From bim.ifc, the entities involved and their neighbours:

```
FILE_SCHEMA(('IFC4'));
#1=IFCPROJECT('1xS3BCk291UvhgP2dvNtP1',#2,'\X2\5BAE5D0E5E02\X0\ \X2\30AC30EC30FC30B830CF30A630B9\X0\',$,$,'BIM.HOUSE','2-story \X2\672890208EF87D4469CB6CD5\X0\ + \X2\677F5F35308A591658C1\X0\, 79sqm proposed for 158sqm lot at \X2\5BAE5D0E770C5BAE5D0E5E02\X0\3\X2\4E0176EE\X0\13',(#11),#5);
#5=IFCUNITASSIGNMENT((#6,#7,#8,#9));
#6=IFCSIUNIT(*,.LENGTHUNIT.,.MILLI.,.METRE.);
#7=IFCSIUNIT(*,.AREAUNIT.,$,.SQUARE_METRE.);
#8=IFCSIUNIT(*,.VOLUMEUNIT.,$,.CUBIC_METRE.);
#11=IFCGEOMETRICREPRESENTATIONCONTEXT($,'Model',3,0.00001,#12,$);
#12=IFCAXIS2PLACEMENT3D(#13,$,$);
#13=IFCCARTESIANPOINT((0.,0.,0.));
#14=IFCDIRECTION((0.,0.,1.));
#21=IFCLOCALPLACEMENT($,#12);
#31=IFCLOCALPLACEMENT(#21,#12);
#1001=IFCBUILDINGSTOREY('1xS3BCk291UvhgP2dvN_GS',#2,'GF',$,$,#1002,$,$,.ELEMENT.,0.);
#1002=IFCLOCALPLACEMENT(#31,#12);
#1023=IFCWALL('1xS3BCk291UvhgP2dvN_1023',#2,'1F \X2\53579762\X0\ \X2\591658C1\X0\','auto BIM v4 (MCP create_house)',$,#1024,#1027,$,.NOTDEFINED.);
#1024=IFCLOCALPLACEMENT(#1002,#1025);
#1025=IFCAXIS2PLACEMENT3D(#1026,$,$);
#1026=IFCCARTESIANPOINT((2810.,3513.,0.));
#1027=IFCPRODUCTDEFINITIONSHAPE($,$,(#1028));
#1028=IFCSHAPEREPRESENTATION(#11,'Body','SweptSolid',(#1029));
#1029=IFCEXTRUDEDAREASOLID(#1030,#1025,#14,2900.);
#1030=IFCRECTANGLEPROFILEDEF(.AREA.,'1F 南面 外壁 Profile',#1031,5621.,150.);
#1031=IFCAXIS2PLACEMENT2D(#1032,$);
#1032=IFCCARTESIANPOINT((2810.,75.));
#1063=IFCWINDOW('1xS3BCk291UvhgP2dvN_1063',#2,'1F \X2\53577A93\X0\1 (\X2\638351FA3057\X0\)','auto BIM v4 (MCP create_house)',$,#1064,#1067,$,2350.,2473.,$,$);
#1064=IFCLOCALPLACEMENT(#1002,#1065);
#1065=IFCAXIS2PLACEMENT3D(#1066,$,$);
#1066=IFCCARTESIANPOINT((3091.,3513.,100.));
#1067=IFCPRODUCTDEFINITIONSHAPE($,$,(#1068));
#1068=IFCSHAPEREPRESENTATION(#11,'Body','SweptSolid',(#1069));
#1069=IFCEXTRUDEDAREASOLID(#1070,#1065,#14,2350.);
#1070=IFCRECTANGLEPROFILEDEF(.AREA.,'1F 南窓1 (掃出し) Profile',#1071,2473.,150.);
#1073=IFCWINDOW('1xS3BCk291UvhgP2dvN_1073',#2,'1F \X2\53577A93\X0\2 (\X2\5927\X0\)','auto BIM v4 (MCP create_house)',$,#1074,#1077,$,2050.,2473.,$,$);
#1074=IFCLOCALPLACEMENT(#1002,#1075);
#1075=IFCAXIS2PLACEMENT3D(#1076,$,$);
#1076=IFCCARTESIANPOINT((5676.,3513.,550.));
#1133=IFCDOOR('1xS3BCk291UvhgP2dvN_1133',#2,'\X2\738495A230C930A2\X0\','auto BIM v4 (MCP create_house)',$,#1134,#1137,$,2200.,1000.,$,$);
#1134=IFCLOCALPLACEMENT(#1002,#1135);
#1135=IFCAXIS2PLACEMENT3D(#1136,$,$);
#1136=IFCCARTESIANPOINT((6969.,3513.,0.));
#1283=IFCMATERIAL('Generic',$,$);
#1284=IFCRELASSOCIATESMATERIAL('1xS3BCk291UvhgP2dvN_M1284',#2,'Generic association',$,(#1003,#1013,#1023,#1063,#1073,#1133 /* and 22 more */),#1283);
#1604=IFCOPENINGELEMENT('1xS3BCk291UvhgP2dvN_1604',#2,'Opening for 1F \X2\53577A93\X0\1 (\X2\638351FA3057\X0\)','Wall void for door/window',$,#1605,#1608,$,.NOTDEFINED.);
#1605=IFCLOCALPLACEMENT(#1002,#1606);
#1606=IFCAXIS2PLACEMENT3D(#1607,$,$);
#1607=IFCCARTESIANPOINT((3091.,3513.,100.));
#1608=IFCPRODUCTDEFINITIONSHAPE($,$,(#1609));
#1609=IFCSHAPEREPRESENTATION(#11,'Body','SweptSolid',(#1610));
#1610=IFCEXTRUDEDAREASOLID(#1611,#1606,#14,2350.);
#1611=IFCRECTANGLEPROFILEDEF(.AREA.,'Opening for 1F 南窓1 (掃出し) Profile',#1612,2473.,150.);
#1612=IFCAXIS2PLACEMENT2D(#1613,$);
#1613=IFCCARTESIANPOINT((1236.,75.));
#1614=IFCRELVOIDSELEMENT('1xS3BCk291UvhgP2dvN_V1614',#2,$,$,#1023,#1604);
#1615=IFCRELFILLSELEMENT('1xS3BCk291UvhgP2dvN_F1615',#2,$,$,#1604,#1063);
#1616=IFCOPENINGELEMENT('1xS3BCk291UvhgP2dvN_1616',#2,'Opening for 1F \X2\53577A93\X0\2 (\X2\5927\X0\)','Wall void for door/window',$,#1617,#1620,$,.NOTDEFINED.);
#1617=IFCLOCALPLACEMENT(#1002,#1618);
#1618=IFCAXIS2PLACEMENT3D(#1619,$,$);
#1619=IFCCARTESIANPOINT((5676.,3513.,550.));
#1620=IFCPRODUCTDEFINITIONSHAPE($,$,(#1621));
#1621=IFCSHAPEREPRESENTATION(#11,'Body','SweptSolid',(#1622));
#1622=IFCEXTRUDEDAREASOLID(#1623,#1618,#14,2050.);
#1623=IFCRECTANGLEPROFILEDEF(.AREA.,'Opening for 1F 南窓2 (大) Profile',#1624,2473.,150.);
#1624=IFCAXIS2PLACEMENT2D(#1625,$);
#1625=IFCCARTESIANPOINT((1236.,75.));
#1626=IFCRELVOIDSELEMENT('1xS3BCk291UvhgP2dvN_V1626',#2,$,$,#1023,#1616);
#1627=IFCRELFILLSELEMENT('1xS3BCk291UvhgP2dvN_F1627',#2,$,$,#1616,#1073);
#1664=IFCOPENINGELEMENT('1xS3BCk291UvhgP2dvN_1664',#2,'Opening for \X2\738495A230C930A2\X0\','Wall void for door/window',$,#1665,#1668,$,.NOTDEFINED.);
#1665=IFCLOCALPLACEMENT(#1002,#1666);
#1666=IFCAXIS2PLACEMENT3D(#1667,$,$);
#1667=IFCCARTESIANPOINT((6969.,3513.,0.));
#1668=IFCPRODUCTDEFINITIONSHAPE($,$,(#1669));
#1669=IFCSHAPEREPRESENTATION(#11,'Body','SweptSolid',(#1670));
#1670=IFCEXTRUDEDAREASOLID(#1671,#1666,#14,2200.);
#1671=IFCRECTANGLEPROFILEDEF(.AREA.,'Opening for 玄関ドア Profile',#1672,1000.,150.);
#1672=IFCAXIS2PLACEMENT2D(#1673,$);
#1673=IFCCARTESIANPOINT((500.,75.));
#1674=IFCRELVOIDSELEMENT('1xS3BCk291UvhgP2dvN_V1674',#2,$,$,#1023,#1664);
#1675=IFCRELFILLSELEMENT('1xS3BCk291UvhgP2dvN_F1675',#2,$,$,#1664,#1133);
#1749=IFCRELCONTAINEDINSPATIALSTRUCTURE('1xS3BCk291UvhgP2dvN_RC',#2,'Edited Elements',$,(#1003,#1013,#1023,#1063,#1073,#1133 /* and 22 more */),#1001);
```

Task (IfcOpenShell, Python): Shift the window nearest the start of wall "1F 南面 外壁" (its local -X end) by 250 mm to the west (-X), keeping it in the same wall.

```python
import ifcopenshell
import ifcopenshell.api.geometry
import ifcopenshell.util.placement

model = ifcopenshell.open("bim.ifc")

window = model.by_guid("1xS3BCk291UvhgP2dvN_1063")
opening = window.FillsVoids[0].RelatingOpeningElement
wall = opening.VoidsElements[0].RelatingBuildingElement

wall_matrix = ifcopenshell.util.placement.get_local_placement(wall.ObjectPlacement)
shift = wall_matrix[:3, 0] * -250.0
before = ifcopenshell.util.placement.get_local_placement(window.ObjectPlacement)[:3, 3].copy()

# The window is not placed relative to its opening, so move both.
for product in (opening, window):
    matrix = ifcopenshell.util.placement.get_local_placement(product.ObjectPlacement)
    matrix[:3, 3] += shift
    ifcopenshell.api.geometry.edit_object_placement(model, product=product, matrix=matrix, is_si=False)

after = ifcopenshell.util.placement.get_local_placement(window.ObjectPlacement)[:3, 3]
print("window moved by", (after - before).round(3) + 0.0)

model.write("bim_rev.ifc")
```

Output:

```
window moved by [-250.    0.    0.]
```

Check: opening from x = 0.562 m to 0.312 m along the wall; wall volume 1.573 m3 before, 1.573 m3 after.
